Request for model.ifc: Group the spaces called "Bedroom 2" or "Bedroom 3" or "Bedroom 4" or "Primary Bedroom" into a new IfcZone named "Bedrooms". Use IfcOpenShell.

First a look at what the model holds.

```python
import ifcopenshell

model = ifcopenshell.open("model.ifc")
print(model.schema)
seen = {}
for space in model.by_type("IfcSpace"):
    seen[space.LongName] = seen.get(space.LongName, 0) + 1
for name, count in sorted(seen.items(), key=str):
    print(count, "x", name)
print("zones:", [z.Name for z in model.by_type("IfcZone")][:20])
```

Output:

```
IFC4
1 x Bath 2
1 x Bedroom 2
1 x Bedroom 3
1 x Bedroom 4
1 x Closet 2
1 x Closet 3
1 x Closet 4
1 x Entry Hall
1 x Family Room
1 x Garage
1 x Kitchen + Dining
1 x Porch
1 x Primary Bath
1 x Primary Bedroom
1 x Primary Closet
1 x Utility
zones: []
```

```python
import ifcopenshell
import ifcopenshell.api.group
import ifcopenshell.api.root

model = ifcopenshell.open("model.ifc")

names = {"Bedroom 2", "Bedroom 3", "Bedroom 4", "Primary Bedroom"}
spaces = [s for s in model.by_type("IfcSpace") if s.LongName in names]

zone = ifcopenshell.api.root.create_entity(model, ifc_class="IfcZone", name="Bedrooms")
ifcopenshell.api.group.assign_group(model, products=spaces, group=zone)
print(len(spaces), "spaces in", zone.Name)

model.write("model_updated.ifc")
```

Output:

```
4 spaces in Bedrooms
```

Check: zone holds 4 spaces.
